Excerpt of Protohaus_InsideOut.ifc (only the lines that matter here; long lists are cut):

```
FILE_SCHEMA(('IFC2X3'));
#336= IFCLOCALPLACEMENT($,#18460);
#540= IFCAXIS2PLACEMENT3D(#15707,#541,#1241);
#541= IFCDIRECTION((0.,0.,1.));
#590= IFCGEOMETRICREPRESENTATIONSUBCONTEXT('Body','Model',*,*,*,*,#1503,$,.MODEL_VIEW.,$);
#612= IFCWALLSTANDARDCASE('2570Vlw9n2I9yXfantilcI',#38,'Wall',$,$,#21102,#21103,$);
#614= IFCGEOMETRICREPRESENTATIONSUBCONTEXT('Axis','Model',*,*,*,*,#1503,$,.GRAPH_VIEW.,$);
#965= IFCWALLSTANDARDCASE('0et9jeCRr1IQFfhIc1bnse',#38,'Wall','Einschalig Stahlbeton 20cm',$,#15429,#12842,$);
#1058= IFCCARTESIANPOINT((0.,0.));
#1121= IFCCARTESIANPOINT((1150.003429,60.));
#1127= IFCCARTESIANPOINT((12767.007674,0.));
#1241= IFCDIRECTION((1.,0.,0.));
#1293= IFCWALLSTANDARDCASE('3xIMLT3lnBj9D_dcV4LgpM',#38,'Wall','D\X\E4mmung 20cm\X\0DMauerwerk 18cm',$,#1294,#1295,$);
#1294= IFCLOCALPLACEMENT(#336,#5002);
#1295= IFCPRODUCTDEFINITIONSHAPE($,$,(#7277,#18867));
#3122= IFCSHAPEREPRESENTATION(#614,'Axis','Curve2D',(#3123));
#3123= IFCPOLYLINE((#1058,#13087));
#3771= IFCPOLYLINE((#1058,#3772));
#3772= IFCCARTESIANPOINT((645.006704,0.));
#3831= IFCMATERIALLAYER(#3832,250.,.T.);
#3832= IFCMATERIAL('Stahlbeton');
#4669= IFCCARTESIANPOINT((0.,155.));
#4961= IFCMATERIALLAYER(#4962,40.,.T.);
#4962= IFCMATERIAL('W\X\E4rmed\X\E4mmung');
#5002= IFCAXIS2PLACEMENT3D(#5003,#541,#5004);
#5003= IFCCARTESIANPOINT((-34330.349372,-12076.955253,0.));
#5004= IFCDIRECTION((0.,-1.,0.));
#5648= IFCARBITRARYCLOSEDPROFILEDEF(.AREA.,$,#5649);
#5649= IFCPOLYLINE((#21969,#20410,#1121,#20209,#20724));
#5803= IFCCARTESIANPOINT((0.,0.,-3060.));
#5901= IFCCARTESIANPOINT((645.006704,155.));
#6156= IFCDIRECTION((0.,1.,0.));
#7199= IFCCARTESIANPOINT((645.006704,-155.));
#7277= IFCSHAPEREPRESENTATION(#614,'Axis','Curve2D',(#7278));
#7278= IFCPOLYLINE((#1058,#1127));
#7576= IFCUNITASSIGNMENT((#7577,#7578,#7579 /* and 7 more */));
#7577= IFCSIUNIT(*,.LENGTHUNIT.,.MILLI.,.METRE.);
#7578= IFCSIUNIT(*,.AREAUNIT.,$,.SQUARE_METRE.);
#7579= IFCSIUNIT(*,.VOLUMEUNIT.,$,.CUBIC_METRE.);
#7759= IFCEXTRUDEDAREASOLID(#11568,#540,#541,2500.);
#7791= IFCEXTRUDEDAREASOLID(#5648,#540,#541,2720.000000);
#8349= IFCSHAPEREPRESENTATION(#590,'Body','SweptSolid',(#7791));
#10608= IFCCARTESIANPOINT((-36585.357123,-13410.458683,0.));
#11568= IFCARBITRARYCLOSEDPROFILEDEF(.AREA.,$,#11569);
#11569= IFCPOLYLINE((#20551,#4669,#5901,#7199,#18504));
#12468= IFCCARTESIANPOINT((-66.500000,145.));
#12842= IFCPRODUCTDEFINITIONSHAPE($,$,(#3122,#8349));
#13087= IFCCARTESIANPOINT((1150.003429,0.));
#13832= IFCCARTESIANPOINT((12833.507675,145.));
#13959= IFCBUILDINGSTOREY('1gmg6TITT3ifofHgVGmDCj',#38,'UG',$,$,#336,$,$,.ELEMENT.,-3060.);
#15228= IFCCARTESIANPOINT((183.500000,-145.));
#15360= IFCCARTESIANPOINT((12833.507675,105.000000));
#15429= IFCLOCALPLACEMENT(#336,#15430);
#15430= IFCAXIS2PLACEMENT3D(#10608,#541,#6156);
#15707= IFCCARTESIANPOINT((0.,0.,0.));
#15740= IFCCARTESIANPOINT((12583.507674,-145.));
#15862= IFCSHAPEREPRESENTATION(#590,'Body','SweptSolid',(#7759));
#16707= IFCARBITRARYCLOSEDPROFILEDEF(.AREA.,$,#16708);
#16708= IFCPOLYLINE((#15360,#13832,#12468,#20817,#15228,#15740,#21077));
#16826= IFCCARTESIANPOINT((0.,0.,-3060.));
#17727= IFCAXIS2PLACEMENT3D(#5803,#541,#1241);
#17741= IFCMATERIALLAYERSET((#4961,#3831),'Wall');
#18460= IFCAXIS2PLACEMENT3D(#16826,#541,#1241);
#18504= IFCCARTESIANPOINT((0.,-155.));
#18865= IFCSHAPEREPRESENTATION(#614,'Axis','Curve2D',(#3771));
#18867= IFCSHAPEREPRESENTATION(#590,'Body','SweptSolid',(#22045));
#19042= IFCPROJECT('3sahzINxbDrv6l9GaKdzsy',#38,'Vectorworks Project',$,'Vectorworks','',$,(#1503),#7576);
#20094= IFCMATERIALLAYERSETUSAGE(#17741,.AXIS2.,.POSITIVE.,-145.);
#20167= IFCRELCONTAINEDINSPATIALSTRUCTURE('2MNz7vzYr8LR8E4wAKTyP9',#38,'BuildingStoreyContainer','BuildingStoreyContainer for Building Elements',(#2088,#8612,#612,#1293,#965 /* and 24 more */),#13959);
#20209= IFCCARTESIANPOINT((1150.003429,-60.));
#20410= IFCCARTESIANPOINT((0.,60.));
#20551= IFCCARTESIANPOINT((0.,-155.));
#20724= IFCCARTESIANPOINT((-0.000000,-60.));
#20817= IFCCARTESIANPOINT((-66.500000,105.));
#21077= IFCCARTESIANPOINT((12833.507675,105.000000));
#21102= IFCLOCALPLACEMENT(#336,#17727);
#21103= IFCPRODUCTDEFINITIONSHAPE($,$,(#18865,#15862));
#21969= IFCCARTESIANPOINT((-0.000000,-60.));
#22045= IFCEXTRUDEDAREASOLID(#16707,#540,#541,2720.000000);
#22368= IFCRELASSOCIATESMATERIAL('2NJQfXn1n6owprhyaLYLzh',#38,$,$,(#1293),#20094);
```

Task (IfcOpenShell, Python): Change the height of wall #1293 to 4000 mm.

```python
import ifcopenshell
import ifcopenshell.geom
import ifcopenshell.util.representation
import ifcopenshell.util.shape
import ifcopenshell.util.unit

model = ifcopenshell.open("Protohaus_InsideOut.ifc")
unit_scale = ifcopenshell.util.unit.calculate_unit_scale(model)
settings = ifcopenshell.geom.settings()


def volume(element):
    """Net volume in cubic metres, openings subtracted."""
    shape = ifcopenshell.geom.create_shape(settings, element)
    return ifcopenshell.util.shape.get_volume(shape.geometry)


wall = model.by_guid("3xIMLT3lnBj9D_dcV4LgpM")
before = volume(wall)

body = ifcopenshell.util.representation.get_representation(wall, "Model", "Body")
solid = body.Items[0]
old_height = solid.Depth
solid.Depth = 4 / unit_scale
after = volume(wall)

print(f"height {old_height:g} -> {solid.Depth:g}, volume {before:.3f} -> {after:.3f} m3")

model.write("Protohaus_InsideOut_edited.ifc")
```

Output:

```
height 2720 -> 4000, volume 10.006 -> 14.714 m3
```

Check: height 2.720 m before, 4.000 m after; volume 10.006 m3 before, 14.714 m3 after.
